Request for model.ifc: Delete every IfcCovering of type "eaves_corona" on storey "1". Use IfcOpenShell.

First a look at what the model holds.

```python
import ifcopenshell
import ifcopenshell.util.element

model = ifcopenshell.open("model.ifc")
print(model.schema)
storey = next(s for s in model.by_type("IfcBuildingStorey") if s.Name == "1")
coverings = [e for e in ifcopenshell.util.element.get_decomposition(storey) if e.is_a("IfcCovering")]
seen = {}
for e in coverings:
    element_type = ifcopenshell.util.element.get_type(e)
    name = element_type.Name if element_type not in (None, e) else None
    seen[name] = seen.get(name, 0) + 1
for name, count in sorted(seen.items(), key=str):
    print(count, "x", name)
```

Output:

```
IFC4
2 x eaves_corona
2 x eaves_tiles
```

```python
import ifcopenshell
import ifcopenshell.api.root
import ifcopenshell.util.element

model = ifcopenshell.open("model.ifc")

storey = next(s for s in model.by_type("IfcBuildingStorey") if s.Name == "1")
coverings = [e for e in ifcopenshell.util.element.get_decomposition(storey) if e.is_a("IfcCovering")]
targets = [e for e in coverings if (t := ifcopenshell.util.element.get_type(e)) not in (None, e) and t.Name == "eaves_corona"]

for e in targets:
    ifcopenshell.api.root.remove_product(model, product=e)
print(len(targets), "removed")

model.write("model_updated.ifc")
```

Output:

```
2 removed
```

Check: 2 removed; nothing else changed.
